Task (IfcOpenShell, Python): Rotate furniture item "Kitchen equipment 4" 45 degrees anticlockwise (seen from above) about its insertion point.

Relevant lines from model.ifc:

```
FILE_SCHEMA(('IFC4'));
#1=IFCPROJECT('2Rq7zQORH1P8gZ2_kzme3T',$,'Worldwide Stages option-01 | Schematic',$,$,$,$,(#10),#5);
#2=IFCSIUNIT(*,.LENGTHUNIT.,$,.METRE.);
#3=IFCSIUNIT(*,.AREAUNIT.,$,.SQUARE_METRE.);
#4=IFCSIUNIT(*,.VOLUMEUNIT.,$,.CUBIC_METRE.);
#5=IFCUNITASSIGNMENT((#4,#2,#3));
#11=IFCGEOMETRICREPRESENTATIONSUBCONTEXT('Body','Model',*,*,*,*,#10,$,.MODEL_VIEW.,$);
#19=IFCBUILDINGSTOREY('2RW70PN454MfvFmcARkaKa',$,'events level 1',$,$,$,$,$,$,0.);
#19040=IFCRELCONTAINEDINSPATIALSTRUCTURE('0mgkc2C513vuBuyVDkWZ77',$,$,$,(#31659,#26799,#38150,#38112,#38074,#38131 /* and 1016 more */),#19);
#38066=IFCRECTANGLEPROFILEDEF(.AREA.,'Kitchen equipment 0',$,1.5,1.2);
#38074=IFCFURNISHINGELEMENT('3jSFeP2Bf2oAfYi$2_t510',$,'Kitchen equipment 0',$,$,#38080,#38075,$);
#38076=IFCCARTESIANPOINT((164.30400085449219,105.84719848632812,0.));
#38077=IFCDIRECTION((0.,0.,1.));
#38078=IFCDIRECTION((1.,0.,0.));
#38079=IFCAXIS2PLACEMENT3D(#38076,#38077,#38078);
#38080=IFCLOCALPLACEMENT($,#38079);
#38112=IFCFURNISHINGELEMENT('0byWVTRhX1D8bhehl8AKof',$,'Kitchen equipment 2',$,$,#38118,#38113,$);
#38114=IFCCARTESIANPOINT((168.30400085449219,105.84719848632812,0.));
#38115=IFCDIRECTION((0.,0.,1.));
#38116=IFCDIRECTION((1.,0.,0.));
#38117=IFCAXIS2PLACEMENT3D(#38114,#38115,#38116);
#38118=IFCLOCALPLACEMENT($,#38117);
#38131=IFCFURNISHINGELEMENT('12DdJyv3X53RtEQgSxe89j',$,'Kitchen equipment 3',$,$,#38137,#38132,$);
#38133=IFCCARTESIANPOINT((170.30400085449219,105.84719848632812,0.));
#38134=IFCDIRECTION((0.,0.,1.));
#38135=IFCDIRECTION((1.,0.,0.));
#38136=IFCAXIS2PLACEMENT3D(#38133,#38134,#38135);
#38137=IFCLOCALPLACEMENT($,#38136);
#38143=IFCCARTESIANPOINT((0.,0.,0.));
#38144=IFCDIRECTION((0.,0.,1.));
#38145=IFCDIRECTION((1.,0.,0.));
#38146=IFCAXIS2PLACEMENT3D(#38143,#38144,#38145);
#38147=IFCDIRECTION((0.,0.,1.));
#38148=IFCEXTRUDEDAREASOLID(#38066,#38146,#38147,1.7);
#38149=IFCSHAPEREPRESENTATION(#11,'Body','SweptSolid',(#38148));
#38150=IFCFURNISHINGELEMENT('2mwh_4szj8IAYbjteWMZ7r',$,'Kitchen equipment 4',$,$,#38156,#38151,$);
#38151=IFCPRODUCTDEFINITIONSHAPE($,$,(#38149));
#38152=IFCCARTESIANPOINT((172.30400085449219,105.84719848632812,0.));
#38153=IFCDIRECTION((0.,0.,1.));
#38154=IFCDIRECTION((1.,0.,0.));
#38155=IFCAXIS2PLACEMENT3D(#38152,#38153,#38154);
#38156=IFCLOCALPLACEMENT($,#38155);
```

```python
import ifcopenshell
import ifcopenshell.api.geometry
import ifcopenshell.util.placement

model = ifcopenshell.open("model.ifc")

item = model.by_guid("2mwh_4szj8IAYbjteWMZ7r")
matrix = ifcopenshell.util.placement.get_local_placement(item.ObjectPlacement)
matrix = matrix @ ifcopenshell.util.placement.rotation(45, "Z")
ifcopenshell.api.geometry.edit_object_placement(model, product=item, matrix=matrix, is_si=False)

print(ifcopenshell.util.placement.get_local_placement(item.ObjectPlacement).round(3) + 0.0)

model.write("model_rev.ifc")
```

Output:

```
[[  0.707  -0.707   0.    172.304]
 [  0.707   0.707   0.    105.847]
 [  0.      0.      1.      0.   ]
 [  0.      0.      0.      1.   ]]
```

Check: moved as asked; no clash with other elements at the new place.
